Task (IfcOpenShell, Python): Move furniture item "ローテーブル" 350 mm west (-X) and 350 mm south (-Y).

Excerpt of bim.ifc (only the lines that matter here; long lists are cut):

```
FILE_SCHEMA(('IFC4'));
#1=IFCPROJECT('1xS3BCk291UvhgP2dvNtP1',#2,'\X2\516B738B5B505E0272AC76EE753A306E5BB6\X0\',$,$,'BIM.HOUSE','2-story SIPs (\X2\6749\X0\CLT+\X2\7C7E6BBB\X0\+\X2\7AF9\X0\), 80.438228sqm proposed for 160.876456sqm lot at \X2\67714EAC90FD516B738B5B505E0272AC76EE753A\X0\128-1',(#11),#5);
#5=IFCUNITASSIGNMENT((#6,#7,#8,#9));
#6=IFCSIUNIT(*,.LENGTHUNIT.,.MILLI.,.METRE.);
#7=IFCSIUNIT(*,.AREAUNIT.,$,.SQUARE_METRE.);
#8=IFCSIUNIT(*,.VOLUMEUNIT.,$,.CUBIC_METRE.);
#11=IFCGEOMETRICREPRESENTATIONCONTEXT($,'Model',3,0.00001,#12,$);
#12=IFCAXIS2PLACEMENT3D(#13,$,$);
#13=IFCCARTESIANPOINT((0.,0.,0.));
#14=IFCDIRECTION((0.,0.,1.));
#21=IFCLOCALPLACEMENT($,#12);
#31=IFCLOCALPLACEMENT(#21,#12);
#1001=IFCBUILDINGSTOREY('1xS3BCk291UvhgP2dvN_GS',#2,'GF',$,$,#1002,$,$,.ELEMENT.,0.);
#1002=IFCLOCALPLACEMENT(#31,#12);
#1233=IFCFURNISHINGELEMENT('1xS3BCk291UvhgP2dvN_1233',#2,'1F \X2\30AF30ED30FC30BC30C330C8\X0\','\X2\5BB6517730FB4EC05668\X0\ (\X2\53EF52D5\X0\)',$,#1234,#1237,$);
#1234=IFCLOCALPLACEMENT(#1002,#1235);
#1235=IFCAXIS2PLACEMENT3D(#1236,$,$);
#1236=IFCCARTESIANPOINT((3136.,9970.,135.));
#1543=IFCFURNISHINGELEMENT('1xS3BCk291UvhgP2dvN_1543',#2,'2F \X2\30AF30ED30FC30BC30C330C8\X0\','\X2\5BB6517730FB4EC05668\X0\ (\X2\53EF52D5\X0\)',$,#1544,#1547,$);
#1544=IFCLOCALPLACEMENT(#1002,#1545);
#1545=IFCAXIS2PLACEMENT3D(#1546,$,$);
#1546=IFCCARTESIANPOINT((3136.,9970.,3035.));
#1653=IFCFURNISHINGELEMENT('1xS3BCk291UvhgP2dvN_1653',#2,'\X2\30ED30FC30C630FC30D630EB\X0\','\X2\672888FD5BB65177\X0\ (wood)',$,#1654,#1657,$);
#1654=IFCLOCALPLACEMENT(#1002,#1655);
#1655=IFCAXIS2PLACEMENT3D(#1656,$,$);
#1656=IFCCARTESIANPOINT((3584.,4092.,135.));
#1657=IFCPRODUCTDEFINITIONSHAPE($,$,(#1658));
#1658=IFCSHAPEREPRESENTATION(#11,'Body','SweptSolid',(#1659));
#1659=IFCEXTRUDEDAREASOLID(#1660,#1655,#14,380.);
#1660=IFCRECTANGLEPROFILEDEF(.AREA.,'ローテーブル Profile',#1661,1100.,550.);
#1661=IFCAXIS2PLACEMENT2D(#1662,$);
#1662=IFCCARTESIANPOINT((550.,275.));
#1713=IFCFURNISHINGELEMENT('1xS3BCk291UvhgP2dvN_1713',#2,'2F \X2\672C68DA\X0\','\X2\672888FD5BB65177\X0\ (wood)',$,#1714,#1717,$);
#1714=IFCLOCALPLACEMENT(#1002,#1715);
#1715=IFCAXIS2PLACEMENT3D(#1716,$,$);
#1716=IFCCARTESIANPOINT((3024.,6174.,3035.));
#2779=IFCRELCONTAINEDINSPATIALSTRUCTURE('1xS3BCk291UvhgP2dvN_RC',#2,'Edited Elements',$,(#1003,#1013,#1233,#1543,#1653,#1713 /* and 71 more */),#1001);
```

```python
import ifcopenshell
import ifcopenshell.api.geometry
import ifcopenshell.util.placement

model = ifcopenshell.open("bim.ifc")

item = model.by_guid("1xS3BCk291UvhgP2dvN_1653")
matrix = ifcopenshell.util.placement.get_local_placement(item.ObjectPlacement)
matrix[0, 3] -= 350.0
matrix[1, 3] -= 350.0
ifcopenshell.api.geometry.edit_object_placement(model, product=item, matrix=matrix, is_si=False)

print(ifcopenshell.util.placement.get_local_placement(item.ObjectPlacement).round(3) + 0.0)

model.write("bim_rev.ifc")
```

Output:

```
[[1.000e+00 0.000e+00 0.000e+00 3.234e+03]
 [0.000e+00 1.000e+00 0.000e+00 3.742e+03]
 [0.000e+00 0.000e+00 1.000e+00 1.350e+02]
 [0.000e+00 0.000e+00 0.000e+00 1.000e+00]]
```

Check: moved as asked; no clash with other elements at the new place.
